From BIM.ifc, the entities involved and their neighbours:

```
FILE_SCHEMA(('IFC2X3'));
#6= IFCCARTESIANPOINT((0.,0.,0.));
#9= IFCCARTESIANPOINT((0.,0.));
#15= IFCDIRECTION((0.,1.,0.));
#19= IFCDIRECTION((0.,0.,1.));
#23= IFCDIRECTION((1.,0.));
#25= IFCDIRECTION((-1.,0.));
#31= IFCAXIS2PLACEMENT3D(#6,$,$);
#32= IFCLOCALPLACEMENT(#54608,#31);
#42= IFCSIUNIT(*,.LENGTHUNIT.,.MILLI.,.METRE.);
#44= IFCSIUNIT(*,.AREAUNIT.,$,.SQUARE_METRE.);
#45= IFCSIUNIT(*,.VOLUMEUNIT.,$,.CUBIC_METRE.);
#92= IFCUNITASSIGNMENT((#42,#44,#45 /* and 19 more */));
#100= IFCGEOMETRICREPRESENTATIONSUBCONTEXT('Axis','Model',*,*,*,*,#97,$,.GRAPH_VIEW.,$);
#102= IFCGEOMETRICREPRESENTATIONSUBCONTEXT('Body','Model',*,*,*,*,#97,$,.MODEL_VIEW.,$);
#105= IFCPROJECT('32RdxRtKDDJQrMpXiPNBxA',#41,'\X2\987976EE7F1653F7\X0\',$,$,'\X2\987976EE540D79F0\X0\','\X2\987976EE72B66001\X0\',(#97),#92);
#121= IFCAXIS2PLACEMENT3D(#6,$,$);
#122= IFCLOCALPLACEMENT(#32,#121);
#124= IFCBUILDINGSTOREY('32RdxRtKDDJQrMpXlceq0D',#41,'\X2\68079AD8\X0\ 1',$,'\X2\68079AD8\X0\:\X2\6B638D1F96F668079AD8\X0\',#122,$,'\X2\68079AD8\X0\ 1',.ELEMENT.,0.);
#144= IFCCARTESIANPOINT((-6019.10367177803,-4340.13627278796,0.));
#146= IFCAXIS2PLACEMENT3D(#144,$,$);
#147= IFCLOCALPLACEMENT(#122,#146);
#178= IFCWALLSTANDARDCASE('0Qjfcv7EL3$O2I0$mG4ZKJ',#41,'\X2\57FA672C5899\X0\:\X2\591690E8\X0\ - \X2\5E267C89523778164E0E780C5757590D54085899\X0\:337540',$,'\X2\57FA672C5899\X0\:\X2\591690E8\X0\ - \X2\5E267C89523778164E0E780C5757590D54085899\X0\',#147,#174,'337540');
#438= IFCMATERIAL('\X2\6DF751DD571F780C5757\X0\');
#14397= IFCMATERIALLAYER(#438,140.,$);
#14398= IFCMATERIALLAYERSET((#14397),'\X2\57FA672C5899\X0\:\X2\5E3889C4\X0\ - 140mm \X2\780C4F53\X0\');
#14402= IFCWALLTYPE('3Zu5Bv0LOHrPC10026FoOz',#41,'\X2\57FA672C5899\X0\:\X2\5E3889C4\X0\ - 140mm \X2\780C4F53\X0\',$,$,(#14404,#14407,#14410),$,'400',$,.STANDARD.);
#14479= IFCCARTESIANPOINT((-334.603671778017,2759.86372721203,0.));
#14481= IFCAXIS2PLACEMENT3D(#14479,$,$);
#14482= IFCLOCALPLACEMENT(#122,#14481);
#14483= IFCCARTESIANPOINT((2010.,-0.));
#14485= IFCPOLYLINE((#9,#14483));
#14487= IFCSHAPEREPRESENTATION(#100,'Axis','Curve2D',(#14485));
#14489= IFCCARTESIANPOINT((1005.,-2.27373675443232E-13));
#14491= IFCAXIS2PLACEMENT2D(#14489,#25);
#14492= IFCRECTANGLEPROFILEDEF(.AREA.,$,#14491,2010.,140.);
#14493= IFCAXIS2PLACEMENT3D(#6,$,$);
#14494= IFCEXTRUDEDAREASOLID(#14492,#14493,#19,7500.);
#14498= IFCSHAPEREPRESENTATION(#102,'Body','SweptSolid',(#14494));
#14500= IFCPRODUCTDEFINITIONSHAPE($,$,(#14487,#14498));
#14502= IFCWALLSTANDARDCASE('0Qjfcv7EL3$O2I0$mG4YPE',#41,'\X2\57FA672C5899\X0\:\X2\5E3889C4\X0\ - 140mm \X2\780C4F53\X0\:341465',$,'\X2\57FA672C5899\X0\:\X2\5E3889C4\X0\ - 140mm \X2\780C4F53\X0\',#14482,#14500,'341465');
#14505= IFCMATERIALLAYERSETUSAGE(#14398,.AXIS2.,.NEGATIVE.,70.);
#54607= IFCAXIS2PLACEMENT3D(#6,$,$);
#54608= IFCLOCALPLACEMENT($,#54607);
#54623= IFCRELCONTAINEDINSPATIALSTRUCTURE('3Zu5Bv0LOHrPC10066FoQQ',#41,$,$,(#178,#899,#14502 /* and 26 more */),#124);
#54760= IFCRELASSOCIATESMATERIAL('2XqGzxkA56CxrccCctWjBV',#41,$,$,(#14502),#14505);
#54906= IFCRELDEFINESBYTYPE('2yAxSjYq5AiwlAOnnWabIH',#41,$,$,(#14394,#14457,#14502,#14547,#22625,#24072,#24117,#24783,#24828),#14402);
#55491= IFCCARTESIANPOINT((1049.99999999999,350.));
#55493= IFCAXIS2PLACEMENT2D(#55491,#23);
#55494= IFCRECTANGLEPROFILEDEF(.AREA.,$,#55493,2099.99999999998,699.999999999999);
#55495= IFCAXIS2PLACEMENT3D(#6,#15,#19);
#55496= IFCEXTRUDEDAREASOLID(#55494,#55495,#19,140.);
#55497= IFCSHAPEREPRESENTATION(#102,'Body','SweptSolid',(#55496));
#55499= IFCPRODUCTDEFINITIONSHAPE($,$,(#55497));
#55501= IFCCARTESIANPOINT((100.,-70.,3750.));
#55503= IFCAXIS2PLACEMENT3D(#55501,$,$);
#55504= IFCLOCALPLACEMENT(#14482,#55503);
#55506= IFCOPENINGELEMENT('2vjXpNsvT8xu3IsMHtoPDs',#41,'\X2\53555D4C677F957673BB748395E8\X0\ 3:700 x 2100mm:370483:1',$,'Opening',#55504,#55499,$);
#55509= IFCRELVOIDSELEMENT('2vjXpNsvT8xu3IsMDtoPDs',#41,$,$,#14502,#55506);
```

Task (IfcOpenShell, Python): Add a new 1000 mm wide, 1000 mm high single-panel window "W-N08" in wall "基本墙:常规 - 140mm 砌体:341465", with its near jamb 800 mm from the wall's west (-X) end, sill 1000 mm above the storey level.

```python
import numpy as np
import ifcopenshell
import ifcopenshell.api.feature
import ifcopenshell.api.geometry
import ifcopenshell.api.root
import ifcopenshell.api.spatial
import ifcopenshell.api.type
import ifcopenshell.geom
import ifcopenshell.util.element
import ifcopenshell.util.placement
import ifcopenshell.util.representation
import ifcopenshell.util.shape
import ifcopenshell.util.unit

model = ifcopenshell.open("BIM.ifc")
unit_scale = ifcopenshell.util.unit.calculate_unit_scale(model)
settings = ifcopenshell.geom.settings()


def volume(element):
    """Net volume in cubic metres, openings subtracted."""
    shape = ifcopenshell.geom.create_shape(settings, element)
    return ifcopenshell.util.shape.get_volume(shape.geometry)


wall = model.by_guid("0Qjfcv7EL3$O2I0$mG4YPE")
storey = ifcopenshell.util.element.get_container(wall, ifc_class="IfcBuildingStorey")
context = ifcopenshell.util.representation.get_context(model, "Model", "Body", "MODEL_VIEW")
before = volume(wall)

width, height, from_end, sill = 1, 1, 0.8, 1  # metres

# The wall runs along its own X axis, and the end named is its -X end.
wall_shape = ifcopenshell.geom.create_shape(settings, wall)
x, y, z = ifcopenshell.util.shape.get_vertices(wall_shape.geometry).T
start = x.min() + from_end
face, thickness = float(y.min()), float(y.max() - y.min())
wall_matrix = ifcopenshell.util.placement.get_local_placement(wall.ObjectPlacement)
level = ifcopenshell.util.placement.get_local_placement(storey.ObjectPlacement)[2, 3]


def in_wall(x, y):
    """Placement at x, y metres in the wall's axes, at sill height."""
    matrix = wall_matrix.copy()
    matrix[:, 3] = wall_matrix @ np.array([x / unit_scale, y / unit_scale, 0.0, 1.0])
    matrix[2, 3] = level + sill / unit_scale
    return matrix


# Opening: a box that overshoots both wall faces by 50 mm.
opening = ifcopenshell.api.root.create_entity(model, ifc_class="IfcOpeningElement")
box = ifcopenshell.api.geometry.add_wall_representation(
    model, context=context, length=width, height=height, thickness=thickness + 0.1
)
ifcopenshell.api.geometry.assign_representation(model, product=opening, representation=box)
ifcopenshell.api.geometry.edit_object_placement(model, product=opening, matrix=in_wall(start, face - 0.05), is_si=False)
ifcopenshell.api.feature.add_feature(model, feature=opening, element=wall)

window = ifcopenshell.api.root.create_entity(model, ifc_class="IfcWindow", name="W-N08")
window.OverallWidth, window.OverallHeight = width / unit_scale, height / unit_scale
body = ifcopenshell.api.geometry.add_window_representation(
    model,
    context=context,
    overall_width=window.OverallWidth,
    overall_height=window.OverallHeight,
    partition_type="SINGLE_PANEL",
)
ifcopenshell.api.geometry.assign_representation(model, product=window, representation=body)
ifcopenshell.api.spatial.assign_container(model, products=[window], relating_structure=storey)
fills = ifcopenshell.api.feature.add_filling(model, opening=opening, element=window)
fills.OwnerHistory = window.OwnerHistory  # required in IFC2X3

# IFC2X3 keeps the operation on the window style.
style = ifcopenshell.api.root.create_entity(model, ifc_class="IfcWindowStyle", name="W-N08")
style.OperationType, style.ConstructionType = "SINGLE_PANEL", "NOTDEFINED"
style.ParameterTakesPrecedence = style.Sizeable = False
ifcopenshell.api.type.assign_type(model, related_objects=[window], relating_type=style)

# Centre the window in the wall's thickness.
ifcopenshell.api.geometry.edit_object_placement(model, product=window, matrix=in_wall(start, face), is_si=False)
window_shape = ifcopenshell.geom.create_shape(settings, window)
depth = ifcopenshell.util.shape.get_vertices(window_shape.geometry)[:, 1]
offset = face + thickness / 2 - (depth.min() + depth.max()) / 2
ifcopenshell.api.geometry.edit_object_placement(model, product=window, matrix=in_wall(start, offset), is_si=False)

after = volume(wall)

print(f"wall volume {before:.3f} -> {after:.3f} m3")

model.write("BIM_rev.ifc")
```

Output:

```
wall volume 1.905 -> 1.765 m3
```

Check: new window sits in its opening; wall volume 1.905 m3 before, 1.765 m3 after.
